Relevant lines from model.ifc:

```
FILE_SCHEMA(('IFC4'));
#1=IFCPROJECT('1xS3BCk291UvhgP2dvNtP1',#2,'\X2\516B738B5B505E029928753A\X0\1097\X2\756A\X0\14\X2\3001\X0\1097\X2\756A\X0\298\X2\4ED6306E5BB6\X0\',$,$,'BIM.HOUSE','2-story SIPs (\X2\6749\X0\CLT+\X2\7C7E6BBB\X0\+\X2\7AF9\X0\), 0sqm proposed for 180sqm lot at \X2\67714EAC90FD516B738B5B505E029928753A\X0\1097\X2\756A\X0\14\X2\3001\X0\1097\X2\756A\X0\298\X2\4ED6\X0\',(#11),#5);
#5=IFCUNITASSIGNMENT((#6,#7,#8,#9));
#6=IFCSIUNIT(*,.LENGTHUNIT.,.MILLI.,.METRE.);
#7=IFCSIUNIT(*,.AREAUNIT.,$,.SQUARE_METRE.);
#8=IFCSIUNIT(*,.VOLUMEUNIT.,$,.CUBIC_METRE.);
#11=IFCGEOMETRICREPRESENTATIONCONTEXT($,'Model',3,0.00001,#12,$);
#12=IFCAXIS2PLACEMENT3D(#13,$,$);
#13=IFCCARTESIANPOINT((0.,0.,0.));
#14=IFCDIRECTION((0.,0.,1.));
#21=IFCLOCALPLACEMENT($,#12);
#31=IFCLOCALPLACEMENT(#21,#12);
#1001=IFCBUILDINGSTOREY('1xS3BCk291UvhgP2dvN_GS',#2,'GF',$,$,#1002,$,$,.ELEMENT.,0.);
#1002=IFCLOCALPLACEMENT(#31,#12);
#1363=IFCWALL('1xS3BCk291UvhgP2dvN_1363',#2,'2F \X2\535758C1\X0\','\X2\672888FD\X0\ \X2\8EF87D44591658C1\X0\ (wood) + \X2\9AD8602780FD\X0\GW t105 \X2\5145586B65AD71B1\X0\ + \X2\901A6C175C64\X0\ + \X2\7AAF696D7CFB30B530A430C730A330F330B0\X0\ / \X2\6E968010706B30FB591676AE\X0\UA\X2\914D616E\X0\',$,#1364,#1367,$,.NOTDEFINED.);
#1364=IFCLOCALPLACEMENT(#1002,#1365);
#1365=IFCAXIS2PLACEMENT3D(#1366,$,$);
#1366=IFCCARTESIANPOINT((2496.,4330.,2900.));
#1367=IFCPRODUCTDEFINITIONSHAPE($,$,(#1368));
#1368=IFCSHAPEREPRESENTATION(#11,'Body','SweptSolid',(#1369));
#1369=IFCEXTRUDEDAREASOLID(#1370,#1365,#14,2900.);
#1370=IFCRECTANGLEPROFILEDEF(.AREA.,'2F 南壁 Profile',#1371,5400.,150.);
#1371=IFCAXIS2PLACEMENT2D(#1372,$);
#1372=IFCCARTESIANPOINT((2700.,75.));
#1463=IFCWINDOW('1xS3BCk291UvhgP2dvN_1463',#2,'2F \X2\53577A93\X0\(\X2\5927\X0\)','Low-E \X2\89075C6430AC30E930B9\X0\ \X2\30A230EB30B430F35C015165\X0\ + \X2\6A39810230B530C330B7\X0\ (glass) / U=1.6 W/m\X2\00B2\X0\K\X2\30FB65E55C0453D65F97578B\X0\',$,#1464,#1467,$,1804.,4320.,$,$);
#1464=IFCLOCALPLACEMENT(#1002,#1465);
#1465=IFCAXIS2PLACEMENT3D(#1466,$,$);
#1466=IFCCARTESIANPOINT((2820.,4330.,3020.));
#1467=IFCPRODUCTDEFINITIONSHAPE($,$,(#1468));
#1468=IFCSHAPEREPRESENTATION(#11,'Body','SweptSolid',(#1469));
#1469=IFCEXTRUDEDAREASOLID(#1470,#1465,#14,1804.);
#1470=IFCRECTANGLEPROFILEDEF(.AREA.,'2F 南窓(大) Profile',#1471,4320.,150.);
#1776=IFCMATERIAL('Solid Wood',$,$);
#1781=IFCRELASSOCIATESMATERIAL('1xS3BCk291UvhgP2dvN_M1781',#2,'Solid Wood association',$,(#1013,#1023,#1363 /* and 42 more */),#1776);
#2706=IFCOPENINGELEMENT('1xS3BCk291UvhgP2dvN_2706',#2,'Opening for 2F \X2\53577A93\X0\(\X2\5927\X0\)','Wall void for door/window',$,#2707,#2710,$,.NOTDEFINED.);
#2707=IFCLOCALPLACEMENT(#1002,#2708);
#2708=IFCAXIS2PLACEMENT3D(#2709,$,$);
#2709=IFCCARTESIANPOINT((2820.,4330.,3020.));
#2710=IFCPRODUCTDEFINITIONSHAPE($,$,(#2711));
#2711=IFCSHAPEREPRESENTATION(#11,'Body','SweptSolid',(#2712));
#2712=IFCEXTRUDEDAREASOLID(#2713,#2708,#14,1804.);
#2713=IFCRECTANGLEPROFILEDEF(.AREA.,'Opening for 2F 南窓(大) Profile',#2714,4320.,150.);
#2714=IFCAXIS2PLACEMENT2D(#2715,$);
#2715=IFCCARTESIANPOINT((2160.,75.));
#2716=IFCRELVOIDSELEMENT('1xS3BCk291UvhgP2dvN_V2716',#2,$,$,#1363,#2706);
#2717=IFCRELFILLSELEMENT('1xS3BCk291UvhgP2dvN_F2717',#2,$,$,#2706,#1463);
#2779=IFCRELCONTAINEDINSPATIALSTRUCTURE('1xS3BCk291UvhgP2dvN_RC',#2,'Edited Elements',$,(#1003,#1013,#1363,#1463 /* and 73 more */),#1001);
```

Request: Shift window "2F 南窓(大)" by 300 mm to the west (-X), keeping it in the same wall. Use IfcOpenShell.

```python
import ifcopenshell
import ifcopenshell.api.geometry
import ifcopenshell.util.placement
import ifcopenshell.util.unit

model = ifcopenshell.open("model.ifc")
unit_scale = ifcopenshell.util.unit.calculate_unit_scale(model)

window = model.by_guid("1xS3BCk291UvhgP2dvN_1463")
opening = window.FillsVoids[0].RelatingOpeningElement
wall = opening.VoidsElements[0].RelatingBuildingElement

wall_matrix = ifcopenshell.util.placement.get_local_placement(wall.ObjectPlacement)
shift = wall_matrix[:3, 0] * -0.3 / unit_scale
before = ifcopenshell.util.placement.get_local_placement(window.ObjectPlacement)[:3, 3].copy()

# The window is not placed relative to its opening, so move both.
for product in (opening, window):
    matrix = ifcopenshell.util.placement.get_local_placement(product.ObjectPlacement)
    matrix[:3, 3] += shift
    ifcopenshell.api.geometry.edit_object_placement(model, product=product, matrix=matrix, is_si=False)

after = ifcopenshell.util.placement.get_local_placement(window.ObjectPlacement)[:3, 3]
print("window moved by", (after - before).round(3) + 0.0)

model.write("model_rev.ifc")
```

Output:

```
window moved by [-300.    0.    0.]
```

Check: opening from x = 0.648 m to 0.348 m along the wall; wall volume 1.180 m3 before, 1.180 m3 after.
